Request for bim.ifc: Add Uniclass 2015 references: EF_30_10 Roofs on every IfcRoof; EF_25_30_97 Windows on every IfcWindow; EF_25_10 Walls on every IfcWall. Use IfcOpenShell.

First a look at what the model holds.

```python
import ifcopenshell

model = ifcopenshell.open("bim.ifc")
print(model.schema)
print("classifications:", [c.Name for c in model.by_type("IfcClassification")])
for ifc_class in ("IfcDoor", "IfcRoof", "IfcStair", "IfcWall", "IfcWindow"):
    print(ifc_class, len(model.by_type(ifc_class)))
```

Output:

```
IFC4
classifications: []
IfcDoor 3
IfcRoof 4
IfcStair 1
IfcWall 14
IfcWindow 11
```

```python
import ifcopenshell
import ifcopenshell.api.classification

model = ifcopenshell.open("bim.ifc")

system = ifcopenshell.api.classification.add_classification(model, classification="Uniclass 2015")

codes = {
    "IfcRoof": ("EF_30_10", "Roofs"),
    "IfcWindow": ("EF_25_30_97", "Windows"),
    "IfcWall": ("EF_25_10", "Walls"),
}
for ifc_class, (code, name) in codes.items():
    products = model.by_type(ifc_class)
    ifcopenshell.api.classification.add_reference(
        model, products=products, classification=system, identification=code, name=name
    )
    print(code, len(products))

model.write("bim-out.ifc")
```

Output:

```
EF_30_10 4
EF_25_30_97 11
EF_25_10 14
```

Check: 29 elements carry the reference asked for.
